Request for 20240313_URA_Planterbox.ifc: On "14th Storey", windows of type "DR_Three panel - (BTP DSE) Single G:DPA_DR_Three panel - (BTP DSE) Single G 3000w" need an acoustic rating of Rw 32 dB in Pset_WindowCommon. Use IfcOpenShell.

First a look at what the model holds.

```python
import ifcopenshell
import ifcopenshell.util.element

model = ifcopenshell.open("20240313_URA_Planterbox.ifc")
print(model.schema)
storey = next(s for s in model.by_type("IfcBuildingStorey") if s.Name == "14th Storey")
windows = [e for e in ifcopenshell.util.element.get_decomposition(storey) if e.is_a("IfcWindow")]
seen = {}
for e in windows:
    element_type = ifcopenshell.util.element.get_type(e)
    key = (element_type.Name if element_type != e and element_type else None, ifcopenshell.util.element.get_pset(e, "Pset_WindowCommon", "AcousticRating"))
    seen[key] = seen.get(key, 0) + 1
for (name, value), count in sorted(seen.items(), key=str):
    print(count, "x", name, "|", value)
```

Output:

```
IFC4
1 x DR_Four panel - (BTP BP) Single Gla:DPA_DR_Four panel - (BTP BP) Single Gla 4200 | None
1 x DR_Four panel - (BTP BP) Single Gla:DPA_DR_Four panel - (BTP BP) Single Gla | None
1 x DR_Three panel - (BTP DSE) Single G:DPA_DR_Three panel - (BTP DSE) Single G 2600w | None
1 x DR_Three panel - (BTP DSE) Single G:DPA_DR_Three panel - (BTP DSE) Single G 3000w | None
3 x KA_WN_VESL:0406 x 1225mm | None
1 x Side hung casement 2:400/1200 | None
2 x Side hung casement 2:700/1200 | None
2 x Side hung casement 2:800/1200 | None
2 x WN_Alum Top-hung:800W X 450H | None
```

```python
import ifcopenshell
import ifcopenshell.api.pset
import ifcopenshell.util.element

model = ifcopenshell.open("20240313_URA_Planterbox.ifc")

storey = next(s for s in model.by_type("IfcBuildingStorey") if s.Name == "14th Storey")
windows = [e for e in ifcopenshell.util.element.get_decomposition(storey) if e.is_a("IfcWindow")]

count = 0
for e in windows:
    element_type = ifcopenshell.util.element.get_type(e)
    if element_type in (None, e) or element_type.Name != "DR_Three panel - (BTP DSE) Single G:DPA_DR_Three panel - (BTP DSE) Single G 3000w":
        continue
    # add_pset returns the element's existing set when there is one.
    pset = ifcopenshell.api.pset.add_pset(model, product=e, name="Pset_WindowCommon")
    ifcopenshell.api.pset.edit_pset(model, pset=pset, properties={"AcousticRating": "Rw 32 dB"})
    count += 1

print(count, "windows updated")

model.write("20240313_URA_Planterbox_rev.ifc")
```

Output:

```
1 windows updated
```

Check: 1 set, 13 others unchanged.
